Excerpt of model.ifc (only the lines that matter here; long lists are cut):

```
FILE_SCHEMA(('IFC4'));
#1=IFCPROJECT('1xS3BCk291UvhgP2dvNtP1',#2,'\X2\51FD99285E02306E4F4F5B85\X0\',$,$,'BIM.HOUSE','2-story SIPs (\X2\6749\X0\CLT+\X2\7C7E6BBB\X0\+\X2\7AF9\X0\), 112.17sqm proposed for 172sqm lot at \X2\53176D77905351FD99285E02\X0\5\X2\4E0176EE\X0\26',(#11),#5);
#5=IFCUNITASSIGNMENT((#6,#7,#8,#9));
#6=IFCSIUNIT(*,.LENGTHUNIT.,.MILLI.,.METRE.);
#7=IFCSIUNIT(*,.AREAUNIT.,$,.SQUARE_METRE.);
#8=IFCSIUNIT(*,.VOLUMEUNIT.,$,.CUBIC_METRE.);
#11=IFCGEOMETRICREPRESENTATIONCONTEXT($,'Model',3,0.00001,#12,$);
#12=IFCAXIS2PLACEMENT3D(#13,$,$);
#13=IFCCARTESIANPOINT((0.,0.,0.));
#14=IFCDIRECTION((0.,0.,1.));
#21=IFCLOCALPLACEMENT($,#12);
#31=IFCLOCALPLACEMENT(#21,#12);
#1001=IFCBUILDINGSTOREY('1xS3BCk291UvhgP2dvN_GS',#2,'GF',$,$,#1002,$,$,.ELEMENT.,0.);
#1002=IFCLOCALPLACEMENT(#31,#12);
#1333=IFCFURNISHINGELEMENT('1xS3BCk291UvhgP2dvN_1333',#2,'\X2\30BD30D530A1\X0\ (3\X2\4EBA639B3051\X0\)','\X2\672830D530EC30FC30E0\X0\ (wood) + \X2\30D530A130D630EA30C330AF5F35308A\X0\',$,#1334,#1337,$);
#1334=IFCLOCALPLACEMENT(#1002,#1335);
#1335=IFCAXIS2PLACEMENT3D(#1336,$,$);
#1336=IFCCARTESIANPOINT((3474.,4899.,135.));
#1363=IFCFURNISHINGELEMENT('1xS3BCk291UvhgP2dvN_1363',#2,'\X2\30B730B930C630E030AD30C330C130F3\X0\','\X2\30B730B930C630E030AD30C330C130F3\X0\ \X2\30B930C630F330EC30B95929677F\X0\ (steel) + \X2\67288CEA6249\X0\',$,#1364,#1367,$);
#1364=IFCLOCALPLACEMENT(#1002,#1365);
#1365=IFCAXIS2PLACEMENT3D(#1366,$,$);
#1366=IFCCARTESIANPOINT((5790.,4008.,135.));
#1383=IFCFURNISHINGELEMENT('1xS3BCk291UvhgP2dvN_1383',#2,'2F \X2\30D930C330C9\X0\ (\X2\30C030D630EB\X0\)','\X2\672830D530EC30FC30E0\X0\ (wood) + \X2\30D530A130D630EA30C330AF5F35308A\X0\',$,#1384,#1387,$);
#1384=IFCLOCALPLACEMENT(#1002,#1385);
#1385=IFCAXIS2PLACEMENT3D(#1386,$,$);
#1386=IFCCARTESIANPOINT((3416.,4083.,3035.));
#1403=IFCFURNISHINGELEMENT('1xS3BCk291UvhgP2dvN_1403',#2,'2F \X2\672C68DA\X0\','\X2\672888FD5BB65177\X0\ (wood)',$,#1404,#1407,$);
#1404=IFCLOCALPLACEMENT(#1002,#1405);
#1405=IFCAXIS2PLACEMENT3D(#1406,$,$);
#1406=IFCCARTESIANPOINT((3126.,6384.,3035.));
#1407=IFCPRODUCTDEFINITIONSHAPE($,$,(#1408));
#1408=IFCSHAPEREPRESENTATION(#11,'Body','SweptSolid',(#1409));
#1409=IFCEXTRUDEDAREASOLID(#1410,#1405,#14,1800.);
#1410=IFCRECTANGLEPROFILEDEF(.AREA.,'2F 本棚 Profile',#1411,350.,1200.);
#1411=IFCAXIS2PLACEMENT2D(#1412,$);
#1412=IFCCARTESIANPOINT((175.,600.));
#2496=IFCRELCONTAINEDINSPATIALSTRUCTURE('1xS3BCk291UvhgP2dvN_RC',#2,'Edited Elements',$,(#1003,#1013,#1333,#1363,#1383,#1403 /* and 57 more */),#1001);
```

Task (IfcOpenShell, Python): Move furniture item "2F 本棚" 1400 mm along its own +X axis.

```python
import ifcopenshell
import ifcopenshell.api.geometry
import ifcopenshell.util.placement
import ifcopenshell.util.unit

model = ifcopenshell.open("model.ifc")
unit_scale = ifcopenshell.util.unit.calculate_unit_scale(model)

item = model.by_guid("1xS3BCk291UvhgP2dvN_1403")
matrix = ifcopenshell.util.placement.get_local_placement(item.ObjectPlacement)
matrix[:3, 3] += matrix[:3, 0] * 1.4 / unit_scale
ifcopenshell.api.geometry.edit_object_placement(model, product=item, matrix=matrix, is_si=False)

print(ifcopenshell.util.placement.get_local_placement(item.ObjectPlacement).round(3) + 0.0)

model.write("model-out.ifc")
```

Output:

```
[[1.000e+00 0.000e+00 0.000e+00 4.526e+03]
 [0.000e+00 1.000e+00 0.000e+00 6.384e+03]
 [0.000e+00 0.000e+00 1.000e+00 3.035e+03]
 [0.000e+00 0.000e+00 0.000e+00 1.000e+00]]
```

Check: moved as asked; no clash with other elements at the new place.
